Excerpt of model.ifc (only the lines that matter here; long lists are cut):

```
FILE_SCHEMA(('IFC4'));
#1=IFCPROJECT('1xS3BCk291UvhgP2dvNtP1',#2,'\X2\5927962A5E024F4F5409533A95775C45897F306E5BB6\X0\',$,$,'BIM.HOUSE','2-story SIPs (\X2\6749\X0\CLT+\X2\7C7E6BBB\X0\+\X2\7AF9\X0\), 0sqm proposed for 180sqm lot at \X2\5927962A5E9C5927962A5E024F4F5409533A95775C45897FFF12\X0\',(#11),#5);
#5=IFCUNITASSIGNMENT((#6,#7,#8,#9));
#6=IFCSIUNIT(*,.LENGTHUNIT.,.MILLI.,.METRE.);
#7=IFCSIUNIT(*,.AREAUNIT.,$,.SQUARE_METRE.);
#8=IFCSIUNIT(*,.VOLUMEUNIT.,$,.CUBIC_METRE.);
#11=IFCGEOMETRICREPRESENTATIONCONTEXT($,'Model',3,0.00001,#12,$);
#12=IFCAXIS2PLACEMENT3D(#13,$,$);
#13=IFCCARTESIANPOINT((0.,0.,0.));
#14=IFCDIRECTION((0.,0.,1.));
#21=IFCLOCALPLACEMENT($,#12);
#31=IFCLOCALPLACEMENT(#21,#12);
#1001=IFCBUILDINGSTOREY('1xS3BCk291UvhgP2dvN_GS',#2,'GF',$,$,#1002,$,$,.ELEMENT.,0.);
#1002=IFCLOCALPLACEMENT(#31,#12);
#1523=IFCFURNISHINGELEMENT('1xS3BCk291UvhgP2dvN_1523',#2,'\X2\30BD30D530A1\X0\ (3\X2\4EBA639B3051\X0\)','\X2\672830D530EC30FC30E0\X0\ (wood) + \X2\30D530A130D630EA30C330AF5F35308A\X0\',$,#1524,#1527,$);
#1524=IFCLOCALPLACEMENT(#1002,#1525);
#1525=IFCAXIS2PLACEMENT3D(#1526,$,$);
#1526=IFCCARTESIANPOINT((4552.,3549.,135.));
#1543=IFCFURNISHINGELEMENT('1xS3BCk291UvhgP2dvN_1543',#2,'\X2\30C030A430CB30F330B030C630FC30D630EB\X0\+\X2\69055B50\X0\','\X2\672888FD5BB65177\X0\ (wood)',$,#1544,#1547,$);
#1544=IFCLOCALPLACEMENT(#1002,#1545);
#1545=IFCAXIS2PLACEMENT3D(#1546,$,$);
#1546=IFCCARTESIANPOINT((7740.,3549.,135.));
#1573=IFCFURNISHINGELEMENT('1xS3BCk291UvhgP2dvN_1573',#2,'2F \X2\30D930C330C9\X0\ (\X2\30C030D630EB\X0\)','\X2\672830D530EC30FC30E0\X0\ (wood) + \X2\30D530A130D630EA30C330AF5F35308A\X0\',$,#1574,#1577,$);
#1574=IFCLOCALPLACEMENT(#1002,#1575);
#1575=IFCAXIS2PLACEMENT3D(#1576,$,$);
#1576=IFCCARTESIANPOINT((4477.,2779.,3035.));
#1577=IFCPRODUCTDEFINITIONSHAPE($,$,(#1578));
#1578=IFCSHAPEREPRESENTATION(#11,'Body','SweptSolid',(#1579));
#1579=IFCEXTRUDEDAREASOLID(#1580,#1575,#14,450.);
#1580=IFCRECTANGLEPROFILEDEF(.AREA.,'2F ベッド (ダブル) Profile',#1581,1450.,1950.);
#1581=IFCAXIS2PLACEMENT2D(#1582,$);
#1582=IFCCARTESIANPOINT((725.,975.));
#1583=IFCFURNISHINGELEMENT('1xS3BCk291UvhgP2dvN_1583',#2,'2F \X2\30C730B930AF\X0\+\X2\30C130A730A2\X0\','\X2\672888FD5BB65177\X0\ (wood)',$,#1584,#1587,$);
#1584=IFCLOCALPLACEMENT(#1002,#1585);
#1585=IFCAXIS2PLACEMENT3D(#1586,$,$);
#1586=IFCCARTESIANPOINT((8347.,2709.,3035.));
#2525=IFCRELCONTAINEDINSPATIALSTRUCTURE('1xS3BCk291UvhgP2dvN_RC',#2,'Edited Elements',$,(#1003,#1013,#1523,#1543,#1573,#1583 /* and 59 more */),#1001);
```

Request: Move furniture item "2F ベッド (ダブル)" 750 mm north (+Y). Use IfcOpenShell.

```python
import ifcopenshell
import ifcopenshell.api.geometry
import ifcopenshell.util.placement
import ifcopenshell.util.unit

model = ifcopenshell.open("model.ifc")
unit_scale = ifcopenshell.util.unit.calculate_unit_scale(model)

item = model.by_guid("1xS3BCk291UvhgP2dvN_1573")
matrix = ifcopenshell.util.placement.get_local_placement(item.ObjectPlacement)
matrix[1, 3] += 0.75 / unit_scale
ifcopenshell.api.geometry.edit_object_placement(model, product=item, matrix=matrix, is_si=False)

print(ifcopenshell.util.placement.get_local_placement(item.ObjectPlacement).round(3) + 0.0)

model.write("model_updated.ifc")
```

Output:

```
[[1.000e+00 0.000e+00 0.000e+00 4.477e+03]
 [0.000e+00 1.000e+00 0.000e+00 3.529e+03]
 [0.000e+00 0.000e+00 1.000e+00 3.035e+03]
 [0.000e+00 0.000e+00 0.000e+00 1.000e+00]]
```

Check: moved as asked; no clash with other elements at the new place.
